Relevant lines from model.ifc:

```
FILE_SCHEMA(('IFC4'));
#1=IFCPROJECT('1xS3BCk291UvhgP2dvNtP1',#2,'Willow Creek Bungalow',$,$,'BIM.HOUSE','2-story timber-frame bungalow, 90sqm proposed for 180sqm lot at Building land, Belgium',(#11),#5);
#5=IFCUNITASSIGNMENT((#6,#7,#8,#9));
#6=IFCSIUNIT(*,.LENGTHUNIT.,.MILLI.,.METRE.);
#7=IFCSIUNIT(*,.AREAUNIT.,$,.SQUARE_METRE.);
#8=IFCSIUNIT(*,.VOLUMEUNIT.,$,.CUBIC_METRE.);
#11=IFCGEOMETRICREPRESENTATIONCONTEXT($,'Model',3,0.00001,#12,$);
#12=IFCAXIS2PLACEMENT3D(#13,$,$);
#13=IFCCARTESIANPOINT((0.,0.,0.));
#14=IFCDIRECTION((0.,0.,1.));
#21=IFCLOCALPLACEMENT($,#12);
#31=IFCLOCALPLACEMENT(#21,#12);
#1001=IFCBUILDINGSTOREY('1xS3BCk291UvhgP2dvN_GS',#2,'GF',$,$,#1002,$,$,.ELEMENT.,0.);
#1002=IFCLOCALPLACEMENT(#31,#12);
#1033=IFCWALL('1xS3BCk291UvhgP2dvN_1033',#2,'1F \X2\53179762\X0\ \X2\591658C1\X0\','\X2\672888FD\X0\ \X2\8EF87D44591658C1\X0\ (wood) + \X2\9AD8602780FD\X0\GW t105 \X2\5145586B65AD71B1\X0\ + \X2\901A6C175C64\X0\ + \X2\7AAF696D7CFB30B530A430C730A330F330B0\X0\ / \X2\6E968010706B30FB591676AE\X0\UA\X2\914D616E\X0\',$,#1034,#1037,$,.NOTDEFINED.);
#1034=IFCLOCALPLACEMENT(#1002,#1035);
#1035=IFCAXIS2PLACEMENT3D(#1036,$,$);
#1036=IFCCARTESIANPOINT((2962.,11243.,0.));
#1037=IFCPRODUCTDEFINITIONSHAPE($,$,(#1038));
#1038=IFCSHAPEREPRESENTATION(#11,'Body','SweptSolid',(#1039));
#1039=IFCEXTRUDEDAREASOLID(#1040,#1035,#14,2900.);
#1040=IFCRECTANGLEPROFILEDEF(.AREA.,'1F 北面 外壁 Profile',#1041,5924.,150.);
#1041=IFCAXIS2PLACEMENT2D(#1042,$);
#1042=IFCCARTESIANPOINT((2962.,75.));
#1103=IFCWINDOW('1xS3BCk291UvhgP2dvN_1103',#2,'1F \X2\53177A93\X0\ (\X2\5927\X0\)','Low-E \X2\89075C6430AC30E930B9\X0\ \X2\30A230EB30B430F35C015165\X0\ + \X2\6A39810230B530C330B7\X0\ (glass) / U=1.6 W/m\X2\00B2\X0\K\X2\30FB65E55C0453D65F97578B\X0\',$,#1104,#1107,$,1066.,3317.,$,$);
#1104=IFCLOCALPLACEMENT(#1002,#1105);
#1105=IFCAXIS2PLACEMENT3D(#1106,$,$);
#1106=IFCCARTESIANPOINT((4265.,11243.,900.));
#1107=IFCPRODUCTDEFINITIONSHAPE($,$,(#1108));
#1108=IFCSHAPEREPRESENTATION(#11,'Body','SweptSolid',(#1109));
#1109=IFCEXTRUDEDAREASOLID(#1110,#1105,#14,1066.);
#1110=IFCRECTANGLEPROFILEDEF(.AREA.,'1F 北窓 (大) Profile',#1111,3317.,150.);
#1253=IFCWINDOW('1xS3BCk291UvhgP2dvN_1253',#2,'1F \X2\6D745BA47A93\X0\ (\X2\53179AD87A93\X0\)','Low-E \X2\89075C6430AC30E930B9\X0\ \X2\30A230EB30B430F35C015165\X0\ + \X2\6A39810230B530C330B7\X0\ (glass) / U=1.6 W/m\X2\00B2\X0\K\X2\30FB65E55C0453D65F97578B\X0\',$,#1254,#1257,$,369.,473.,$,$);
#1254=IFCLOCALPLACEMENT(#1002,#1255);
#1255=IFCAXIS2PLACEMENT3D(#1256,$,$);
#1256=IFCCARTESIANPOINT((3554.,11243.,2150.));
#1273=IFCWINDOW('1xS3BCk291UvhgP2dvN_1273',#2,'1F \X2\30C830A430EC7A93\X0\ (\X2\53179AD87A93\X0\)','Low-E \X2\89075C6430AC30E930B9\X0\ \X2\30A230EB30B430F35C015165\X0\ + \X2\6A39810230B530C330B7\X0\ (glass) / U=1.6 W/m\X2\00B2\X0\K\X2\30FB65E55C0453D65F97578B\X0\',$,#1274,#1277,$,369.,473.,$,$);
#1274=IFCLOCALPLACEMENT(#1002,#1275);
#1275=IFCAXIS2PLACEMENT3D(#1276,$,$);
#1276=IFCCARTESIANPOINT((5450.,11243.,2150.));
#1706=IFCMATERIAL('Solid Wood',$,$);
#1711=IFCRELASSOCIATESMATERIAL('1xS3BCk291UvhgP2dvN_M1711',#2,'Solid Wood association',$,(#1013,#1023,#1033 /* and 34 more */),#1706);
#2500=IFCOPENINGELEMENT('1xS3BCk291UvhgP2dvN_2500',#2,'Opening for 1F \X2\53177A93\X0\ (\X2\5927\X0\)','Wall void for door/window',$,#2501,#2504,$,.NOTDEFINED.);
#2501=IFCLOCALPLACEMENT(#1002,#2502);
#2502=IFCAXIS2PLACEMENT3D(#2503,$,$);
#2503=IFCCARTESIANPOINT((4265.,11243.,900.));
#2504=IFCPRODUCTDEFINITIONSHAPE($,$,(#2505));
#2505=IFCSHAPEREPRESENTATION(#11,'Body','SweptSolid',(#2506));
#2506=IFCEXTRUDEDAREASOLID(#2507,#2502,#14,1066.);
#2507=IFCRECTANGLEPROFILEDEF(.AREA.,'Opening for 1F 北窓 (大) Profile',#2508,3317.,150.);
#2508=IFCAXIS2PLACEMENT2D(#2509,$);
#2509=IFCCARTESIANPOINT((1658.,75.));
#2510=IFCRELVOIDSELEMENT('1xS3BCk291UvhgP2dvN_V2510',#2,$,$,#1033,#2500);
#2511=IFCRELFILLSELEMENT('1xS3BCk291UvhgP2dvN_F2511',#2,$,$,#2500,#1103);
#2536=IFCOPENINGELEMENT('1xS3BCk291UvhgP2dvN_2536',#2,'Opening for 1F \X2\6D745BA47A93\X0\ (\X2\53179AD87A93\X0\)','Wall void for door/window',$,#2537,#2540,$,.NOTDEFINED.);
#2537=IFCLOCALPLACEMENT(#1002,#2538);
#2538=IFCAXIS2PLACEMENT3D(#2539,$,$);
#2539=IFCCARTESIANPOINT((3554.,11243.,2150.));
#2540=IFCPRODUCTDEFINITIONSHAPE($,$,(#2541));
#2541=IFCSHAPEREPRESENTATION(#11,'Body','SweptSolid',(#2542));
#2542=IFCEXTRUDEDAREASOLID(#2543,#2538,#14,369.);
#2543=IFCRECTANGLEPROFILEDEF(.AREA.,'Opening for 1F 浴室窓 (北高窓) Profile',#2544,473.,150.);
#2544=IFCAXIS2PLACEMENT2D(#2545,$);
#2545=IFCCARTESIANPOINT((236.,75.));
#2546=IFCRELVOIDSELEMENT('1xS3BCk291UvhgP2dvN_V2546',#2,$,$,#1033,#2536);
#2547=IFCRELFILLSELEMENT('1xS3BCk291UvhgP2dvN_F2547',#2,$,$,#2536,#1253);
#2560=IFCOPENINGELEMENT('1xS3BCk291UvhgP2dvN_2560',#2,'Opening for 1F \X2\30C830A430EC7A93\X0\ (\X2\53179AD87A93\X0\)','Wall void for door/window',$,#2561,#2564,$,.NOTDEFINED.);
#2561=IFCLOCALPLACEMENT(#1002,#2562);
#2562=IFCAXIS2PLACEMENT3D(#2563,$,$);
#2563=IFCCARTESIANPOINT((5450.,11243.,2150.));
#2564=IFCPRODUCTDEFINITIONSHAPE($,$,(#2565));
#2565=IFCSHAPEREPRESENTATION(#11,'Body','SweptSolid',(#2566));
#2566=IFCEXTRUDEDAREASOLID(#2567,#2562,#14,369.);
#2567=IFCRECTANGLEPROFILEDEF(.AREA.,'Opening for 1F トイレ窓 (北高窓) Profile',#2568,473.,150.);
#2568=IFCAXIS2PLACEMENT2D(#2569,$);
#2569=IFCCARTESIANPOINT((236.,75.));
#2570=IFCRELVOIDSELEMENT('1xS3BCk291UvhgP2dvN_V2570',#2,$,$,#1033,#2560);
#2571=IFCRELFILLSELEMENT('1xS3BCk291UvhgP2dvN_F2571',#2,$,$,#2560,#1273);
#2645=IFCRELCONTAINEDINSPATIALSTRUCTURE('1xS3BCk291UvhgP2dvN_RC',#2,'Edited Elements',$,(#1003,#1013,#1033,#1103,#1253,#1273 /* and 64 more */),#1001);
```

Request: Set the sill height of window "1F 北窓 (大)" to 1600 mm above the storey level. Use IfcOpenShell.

```python
import numpy as np
import ifcopenshell
import ifcopenshell.api.geometry
import ifcopenshell.geom
import ifcopenshell.util.element
import ifcopenshell.util.placement
import ifcopenshell.util.shape
import ifcopenshell.util.unit

model = ifcopenshell.open("model.ifc")
unit_scale = ifcopenshell.util.unit.calculate_unit_scale(model)

window = model.by_id(1103)
opening = window.FillsVoids[0].RelatingOpeningElement
storey = ifcopenshell.util.element.get_container(window, ifc_class="IfcBuildingStorey")
level = ifcopenshell.util.placement.get_local_placement(storey.ObjectPlacement)[2, 3]

# The opening's origin need not be at the sill, so measure its lowest point.
shape = ifcopenshell.geom.create_shape(ifcopenshell.geom.settings(), opening)
bottom = ifcopenshell.util.shape.get_shape_bottom_elevation(shape, shape.geometry) / unit_scale
dz = level + 1600.0 - bottom

shift = np.array([0.0, 0.0, dz])
# The window is not placed relative to its opening, so move both.
for product in (opening, window):
    matrix = ifcopenshell.util.placement.get_local_placement(product.ObjectPlacement)
    matrix[:3, 3] += shift
    ifcopenshell.api.geometry.edit_object_placement(model, product=product, matrix=matrix, is_si=False)

print(f"moved by {dz * unit_scale:+.3f} m")

model.write("model_updated.ifc")
```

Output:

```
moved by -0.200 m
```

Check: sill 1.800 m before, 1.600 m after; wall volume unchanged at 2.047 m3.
